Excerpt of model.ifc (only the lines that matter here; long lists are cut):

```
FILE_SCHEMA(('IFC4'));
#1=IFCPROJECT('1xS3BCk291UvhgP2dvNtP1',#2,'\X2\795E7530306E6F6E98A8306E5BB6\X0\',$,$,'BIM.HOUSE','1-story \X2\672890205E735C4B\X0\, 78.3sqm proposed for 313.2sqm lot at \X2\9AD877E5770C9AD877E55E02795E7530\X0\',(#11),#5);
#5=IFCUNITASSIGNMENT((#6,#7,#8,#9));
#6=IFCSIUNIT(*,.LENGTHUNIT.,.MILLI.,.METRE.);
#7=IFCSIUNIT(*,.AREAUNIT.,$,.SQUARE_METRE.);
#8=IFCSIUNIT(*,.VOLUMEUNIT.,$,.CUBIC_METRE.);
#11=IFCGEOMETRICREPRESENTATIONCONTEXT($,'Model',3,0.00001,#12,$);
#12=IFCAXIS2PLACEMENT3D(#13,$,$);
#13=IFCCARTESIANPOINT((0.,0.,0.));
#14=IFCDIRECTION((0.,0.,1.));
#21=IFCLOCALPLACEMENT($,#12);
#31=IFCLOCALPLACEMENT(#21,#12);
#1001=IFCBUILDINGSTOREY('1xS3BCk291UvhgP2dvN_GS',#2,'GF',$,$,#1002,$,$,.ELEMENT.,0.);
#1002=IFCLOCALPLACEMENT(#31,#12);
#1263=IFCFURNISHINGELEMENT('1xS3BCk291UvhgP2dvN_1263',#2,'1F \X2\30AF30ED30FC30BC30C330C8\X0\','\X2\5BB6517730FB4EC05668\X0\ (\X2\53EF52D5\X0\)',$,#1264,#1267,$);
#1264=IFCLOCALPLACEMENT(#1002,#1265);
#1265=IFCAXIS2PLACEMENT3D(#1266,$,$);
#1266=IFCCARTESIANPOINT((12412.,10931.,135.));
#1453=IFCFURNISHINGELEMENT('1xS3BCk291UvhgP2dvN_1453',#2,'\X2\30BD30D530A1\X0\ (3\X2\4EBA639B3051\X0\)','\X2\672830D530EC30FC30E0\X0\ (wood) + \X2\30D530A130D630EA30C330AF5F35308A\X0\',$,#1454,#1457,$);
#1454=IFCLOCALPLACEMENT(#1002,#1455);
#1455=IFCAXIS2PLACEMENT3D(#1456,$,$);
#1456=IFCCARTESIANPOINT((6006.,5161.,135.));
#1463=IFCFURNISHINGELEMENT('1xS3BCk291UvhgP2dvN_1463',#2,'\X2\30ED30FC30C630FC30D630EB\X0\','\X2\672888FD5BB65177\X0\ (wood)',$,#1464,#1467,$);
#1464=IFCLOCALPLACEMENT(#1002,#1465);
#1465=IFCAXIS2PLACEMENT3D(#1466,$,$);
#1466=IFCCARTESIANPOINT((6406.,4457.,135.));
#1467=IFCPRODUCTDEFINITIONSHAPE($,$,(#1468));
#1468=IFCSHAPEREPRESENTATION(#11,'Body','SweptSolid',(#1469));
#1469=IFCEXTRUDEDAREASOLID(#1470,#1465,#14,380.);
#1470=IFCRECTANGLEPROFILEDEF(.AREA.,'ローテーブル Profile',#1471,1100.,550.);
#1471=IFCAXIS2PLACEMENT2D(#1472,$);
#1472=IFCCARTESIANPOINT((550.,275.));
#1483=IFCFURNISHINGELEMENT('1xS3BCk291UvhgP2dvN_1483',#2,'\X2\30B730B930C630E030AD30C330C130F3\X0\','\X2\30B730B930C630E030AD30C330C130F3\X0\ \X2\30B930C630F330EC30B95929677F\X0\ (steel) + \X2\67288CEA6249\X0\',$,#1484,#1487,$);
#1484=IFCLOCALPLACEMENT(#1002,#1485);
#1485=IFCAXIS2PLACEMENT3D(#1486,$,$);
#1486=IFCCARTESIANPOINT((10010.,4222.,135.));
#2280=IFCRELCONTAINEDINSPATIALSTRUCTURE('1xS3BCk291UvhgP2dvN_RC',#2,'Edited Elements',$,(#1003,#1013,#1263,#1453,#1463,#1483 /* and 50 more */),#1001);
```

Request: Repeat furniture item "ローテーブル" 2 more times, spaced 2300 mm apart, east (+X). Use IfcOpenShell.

```python
import numpy as np
import ifcopenshell
import ifcopenshell.api.geometry
import ifcopenshell.api.root
import ifcopenshell.util.element
import ifcopenshell.util.placement
import ifcopenshell.util.unit

model = ifcopenshell.open("model.ifc")
unit_scale = ifcopenshell.util.unit.calculate_unit_scale(model)


def reuse_history(source, copy):
    """copy_class also copies each property set's owner history, people and application; keep the originals."""
    for rel in copy.IsDefinedBy:
        if rel.is_a("IfcRelDefinesByProperties") and (history := rel.RelatingPropertyDefinition.OwnerHistory):
            rel.RelatingPropertyDefinition.OwnerHistory = source.OwnerHistory
            ifcopenshell.util.element.remove_deep2(model, history)


source = model.by_id(1463)
base = ifcopenshell.util.placement.get_local_placement(source.ObjectPlacement)
step = np.array([1.0, 0.0, 0.0]) * 2.3 / unit_scale

for i in range(1, 3):
    copy = ifcopenshell.api.root.copy_class(model, product=source)
    copy.Representation = ifcopenshell.util.element.copy_deep(
        model, source.Representation, exclude=["IfcGeometricRepresentationContext", "IfcRepresentationMap"]
    )
    reuse_history(source, copy)
    matrix = base.copy()
    matrix[:3, 3] += i * step
    print("added at", matrix[:3, 3].round(3) + 0.0)
    ifcopenshell.api.geometry.edit_object_placement(model, product=copy, matrix=matrix, is_si=False)

model.write("model_updated.ifc")
```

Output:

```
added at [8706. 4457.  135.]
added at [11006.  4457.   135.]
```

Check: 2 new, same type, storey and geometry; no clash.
